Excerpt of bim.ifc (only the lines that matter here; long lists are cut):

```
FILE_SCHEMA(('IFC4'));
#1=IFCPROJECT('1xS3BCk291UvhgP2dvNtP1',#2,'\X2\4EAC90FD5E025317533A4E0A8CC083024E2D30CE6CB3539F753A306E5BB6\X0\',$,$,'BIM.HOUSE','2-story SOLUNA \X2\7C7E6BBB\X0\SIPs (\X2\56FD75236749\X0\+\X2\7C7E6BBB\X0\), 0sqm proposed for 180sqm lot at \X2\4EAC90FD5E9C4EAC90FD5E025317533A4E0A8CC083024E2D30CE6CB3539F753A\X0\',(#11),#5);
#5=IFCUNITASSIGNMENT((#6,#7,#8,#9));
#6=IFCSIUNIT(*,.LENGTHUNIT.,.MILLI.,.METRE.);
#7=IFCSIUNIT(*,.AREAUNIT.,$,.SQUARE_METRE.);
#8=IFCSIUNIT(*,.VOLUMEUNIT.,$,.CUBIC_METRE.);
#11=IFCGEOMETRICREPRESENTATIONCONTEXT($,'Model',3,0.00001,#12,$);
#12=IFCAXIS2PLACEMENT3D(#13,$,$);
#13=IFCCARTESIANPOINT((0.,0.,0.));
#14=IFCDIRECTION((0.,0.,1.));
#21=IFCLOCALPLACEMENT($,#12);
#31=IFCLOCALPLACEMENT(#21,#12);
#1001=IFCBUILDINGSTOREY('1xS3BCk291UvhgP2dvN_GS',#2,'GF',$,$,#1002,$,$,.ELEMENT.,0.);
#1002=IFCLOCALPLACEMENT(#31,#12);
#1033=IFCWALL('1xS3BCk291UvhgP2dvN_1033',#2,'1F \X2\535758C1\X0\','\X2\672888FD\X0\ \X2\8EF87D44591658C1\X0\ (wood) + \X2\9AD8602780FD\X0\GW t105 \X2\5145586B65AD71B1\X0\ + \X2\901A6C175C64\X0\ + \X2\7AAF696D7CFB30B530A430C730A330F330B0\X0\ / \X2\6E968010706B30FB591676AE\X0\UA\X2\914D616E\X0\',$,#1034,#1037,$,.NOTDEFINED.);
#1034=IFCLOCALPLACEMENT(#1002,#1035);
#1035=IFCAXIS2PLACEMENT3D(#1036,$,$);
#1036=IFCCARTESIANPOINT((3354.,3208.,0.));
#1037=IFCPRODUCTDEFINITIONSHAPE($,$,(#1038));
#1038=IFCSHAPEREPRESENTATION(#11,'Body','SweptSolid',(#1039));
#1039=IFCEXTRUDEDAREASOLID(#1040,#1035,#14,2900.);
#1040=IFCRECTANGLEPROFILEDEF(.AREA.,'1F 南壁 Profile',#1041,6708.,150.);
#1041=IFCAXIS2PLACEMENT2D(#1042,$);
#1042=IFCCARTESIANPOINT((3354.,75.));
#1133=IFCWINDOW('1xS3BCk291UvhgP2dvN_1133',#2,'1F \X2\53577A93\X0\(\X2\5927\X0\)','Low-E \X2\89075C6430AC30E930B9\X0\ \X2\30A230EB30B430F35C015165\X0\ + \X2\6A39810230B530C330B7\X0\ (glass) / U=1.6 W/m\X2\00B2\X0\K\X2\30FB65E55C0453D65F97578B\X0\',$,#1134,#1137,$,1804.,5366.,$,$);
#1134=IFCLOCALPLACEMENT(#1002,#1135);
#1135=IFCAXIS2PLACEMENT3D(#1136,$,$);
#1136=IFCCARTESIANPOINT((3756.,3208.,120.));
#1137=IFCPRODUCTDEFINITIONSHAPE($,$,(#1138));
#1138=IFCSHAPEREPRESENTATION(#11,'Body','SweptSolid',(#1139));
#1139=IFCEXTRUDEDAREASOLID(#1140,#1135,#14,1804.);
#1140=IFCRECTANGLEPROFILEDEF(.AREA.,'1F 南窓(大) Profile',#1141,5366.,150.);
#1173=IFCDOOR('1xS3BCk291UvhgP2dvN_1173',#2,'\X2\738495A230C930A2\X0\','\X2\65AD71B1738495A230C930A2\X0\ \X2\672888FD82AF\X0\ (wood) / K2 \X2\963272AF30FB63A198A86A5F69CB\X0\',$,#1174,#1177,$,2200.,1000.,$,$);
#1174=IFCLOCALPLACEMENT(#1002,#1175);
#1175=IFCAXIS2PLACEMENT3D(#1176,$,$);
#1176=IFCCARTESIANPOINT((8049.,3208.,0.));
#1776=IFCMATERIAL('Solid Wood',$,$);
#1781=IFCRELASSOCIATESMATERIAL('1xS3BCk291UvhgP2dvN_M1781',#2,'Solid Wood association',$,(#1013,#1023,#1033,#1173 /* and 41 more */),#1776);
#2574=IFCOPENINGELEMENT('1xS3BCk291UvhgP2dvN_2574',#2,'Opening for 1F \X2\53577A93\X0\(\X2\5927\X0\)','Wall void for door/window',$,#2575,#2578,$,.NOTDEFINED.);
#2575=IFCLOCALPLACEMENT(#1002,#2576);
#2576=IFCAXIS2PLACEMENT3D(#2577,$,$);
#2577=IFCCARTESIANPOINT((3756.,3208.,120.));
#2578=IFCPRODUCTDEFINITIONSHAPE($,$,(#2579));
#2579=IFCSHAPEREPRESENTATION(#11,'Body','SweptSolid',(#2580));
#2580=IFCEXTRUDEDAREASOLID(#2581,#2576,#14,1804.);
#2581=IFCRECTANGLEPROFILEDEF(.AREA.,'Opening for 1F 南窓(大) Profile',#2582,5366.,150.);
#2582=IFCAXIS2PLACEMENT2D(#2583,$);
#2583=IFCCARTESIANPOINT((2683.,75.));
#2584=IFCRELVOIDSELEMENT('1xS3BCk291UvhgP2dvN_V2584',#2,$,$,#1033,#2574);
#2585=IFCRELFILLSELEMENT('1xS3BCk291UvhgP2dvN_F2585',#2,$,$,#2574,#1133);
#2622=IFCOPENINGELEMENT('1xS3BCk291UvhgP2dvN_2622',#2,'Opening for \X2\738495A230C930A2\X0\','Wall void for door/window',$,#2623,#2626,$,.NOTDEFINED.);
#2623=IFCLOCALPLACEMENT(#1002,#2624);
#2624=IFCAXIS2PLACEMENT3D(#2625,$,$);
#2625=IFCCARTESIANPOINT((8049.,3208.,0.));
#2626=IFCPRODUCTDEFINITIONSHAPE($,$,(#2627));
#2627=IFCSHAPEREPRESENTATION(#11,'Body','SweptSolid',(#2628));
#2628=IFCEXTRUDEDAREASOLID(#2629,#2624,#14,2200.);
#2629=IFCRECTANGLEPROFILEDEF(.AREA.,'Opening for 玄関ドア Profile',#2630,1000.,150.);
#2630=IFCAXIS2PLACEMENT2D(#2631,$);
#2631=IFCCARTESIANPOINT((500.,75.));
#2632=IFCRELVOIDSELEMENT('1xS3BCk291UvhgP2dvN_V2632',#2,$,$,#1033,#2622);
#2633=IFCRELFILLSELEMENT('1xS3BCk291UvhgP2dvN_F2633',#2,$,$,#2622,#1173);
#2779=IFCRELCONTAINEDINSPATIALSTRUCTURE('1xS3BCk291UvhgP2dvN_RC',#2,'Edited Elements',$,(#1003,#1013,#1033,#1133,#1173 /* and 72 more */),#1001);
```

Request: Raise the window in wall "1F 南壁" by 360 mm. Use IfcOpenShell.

```python
import numpy as np
import ifcopenshell
import ifcopenshell.api.geometry
import ifcopenshell.util.placement
import ifcopenshell.util.unit

model = ifcopenshell.open("bim.ifc")
unit_scale = ifcopenshell.util.unit.calculate_unit_scale(model)

window = model.by_guid("1xS3BCk291UvhgP2dvN_1133")
opening = window.FillsVoids[0].RelatingOpeningElement
dz = 0.36 / unit_scale

shift = np.array([0.0, 0.0, dz])
# The window is not placed relative to its opening, so move both.
for product in (opening, window):
    matrix = ifcopenshell.util.placement.get_local_placement(product.ObjectPlacement)
    matrix[:3, 3] += shift
    ifcopenshell.api.geometry.edit_object_placement(model, product=product, matrix=matrix, is_si=False)

print(f"moved by {dz * unit_scale:+.3f} m")

model.write("bim_rev.ifc")
```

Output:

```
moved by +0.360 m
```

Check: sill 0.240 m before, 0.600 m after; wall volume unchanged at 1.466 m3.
